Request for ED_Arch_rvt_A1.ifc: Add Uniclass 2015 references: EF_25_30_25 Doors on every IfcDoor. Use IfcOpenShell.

First a look at what the model holds.

```python
import ifcopenshell

model = ifcopenshell.open("ED_Arch_rvt_A1.ifc")
print(model.schema)
print("classifications:", [c.Name for c in model.by_type("IfcClassification")])
for ifc_class in ("IfcDoor", "IfcRoof", "IfcStair", "IfcWall", "IfcWindow"):
    print(ifc_class, len(model.by_type(ifc_class)))
```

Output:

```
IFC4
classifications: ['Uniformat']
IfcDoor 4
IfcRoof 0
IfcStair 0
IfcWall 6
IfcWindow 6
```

```python
import ifcopenshell
import ifcopenshell.api.classification

model = ifcopenshell.open("ED_Arch_rvt_A1.ifc")

system = ifcopenshell.api.classification.add_classification(model, classification="Uniclass 2015")

codes = {
    "IfcDoor": ("EF_25_30_25", "Doors"),
}
for ifc_class, (code, name) in codes.items():
    products = model.by_type(ifc_class)
    ifcopenshell.api.classification.add_reference(
        model, products=products, classification=system, identification=code, name=name
    )
    print(code, len(products))

model.write("ED_Arch_rvt_A1_edited.ifc")
```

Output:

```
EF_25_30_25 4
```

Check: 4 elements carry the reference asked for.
